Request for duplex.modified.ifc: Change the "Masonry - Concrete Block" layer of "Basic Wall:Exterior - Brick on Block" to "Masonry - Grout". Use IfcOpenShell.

First a look at what the model holds.

```python
import ifcopenshell
import ifcopenshell.util.element

model = ifcopenshell.open("duplex.modified.ifc")
print(model.schema)
for layer_set in model.by_type("IfcMaterialLayerSet"):
    if layer_set.LayerSetName == "Basic Wall:Exterior - Brick on Block":
        for layer in layer_set.MaterialLayers:
            print(layer.id(), layer.Material and layer.Material.Name, layer.LayerThickness, sep=" | ")
        print(len(ifcopenshell.util.element.get_elements_by_material(model, layer_set)), "elements and types use it")
print(sorted(m.Name for m in model.by_type("IfcMaterial") if m.Name)[:60])
```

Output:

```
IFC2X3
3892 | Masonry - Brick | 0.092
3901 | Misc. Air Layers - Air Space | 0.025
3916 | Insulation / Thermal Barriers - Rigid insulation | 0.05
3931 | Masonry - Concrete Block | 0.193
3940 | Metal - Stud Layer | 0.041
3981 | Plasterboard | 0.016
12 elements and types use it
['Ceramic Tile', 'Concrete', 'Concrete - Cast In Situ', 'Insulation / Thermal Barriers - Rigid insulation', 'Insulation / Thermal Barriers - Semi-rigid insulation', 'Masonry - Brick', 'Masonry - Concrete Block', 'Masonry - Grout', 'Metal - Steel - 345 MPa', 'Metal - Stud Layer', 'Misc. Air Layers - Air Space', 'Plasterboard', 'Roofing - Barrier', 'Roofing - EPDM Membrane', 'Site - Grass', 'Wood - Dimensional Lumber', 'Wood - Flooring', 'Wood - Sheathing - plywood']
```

```python
import ifcopenshell
import ifcopenshell.api.material

model = ifcopenshell.open("duplex.modified.ifc")

layer_set = next(s for s in model.by_type("IfcMaterialLayerSet") if s.LayerSetName == "Basic Wall:Exterior - Brick on Block")
layer = next(l for l in layer_set.MaterialLayers if l.Material and l.Material.Name == "Masonry - Concrete Block")
material = next(m for m in model.by_type("IfcMaterial") if m.Name == "Masonry - Grout")

# Point this one layer at the other material; renaming the old one would change it everywhere.
ifcopenshell.api.material.edit_layer(model, layer=layer, attributes={}, material=material)

print([l.Material.Name if l.Material else None for l in layer_set.MaterialLayers])

model.write("duplex.modified_edited.ifc")
```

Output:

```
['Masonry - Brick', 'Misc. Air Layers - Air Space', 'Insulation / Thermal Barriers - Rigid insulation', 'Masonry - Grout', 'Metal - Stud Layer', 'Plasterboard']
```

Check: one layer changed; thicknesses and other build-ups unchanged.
